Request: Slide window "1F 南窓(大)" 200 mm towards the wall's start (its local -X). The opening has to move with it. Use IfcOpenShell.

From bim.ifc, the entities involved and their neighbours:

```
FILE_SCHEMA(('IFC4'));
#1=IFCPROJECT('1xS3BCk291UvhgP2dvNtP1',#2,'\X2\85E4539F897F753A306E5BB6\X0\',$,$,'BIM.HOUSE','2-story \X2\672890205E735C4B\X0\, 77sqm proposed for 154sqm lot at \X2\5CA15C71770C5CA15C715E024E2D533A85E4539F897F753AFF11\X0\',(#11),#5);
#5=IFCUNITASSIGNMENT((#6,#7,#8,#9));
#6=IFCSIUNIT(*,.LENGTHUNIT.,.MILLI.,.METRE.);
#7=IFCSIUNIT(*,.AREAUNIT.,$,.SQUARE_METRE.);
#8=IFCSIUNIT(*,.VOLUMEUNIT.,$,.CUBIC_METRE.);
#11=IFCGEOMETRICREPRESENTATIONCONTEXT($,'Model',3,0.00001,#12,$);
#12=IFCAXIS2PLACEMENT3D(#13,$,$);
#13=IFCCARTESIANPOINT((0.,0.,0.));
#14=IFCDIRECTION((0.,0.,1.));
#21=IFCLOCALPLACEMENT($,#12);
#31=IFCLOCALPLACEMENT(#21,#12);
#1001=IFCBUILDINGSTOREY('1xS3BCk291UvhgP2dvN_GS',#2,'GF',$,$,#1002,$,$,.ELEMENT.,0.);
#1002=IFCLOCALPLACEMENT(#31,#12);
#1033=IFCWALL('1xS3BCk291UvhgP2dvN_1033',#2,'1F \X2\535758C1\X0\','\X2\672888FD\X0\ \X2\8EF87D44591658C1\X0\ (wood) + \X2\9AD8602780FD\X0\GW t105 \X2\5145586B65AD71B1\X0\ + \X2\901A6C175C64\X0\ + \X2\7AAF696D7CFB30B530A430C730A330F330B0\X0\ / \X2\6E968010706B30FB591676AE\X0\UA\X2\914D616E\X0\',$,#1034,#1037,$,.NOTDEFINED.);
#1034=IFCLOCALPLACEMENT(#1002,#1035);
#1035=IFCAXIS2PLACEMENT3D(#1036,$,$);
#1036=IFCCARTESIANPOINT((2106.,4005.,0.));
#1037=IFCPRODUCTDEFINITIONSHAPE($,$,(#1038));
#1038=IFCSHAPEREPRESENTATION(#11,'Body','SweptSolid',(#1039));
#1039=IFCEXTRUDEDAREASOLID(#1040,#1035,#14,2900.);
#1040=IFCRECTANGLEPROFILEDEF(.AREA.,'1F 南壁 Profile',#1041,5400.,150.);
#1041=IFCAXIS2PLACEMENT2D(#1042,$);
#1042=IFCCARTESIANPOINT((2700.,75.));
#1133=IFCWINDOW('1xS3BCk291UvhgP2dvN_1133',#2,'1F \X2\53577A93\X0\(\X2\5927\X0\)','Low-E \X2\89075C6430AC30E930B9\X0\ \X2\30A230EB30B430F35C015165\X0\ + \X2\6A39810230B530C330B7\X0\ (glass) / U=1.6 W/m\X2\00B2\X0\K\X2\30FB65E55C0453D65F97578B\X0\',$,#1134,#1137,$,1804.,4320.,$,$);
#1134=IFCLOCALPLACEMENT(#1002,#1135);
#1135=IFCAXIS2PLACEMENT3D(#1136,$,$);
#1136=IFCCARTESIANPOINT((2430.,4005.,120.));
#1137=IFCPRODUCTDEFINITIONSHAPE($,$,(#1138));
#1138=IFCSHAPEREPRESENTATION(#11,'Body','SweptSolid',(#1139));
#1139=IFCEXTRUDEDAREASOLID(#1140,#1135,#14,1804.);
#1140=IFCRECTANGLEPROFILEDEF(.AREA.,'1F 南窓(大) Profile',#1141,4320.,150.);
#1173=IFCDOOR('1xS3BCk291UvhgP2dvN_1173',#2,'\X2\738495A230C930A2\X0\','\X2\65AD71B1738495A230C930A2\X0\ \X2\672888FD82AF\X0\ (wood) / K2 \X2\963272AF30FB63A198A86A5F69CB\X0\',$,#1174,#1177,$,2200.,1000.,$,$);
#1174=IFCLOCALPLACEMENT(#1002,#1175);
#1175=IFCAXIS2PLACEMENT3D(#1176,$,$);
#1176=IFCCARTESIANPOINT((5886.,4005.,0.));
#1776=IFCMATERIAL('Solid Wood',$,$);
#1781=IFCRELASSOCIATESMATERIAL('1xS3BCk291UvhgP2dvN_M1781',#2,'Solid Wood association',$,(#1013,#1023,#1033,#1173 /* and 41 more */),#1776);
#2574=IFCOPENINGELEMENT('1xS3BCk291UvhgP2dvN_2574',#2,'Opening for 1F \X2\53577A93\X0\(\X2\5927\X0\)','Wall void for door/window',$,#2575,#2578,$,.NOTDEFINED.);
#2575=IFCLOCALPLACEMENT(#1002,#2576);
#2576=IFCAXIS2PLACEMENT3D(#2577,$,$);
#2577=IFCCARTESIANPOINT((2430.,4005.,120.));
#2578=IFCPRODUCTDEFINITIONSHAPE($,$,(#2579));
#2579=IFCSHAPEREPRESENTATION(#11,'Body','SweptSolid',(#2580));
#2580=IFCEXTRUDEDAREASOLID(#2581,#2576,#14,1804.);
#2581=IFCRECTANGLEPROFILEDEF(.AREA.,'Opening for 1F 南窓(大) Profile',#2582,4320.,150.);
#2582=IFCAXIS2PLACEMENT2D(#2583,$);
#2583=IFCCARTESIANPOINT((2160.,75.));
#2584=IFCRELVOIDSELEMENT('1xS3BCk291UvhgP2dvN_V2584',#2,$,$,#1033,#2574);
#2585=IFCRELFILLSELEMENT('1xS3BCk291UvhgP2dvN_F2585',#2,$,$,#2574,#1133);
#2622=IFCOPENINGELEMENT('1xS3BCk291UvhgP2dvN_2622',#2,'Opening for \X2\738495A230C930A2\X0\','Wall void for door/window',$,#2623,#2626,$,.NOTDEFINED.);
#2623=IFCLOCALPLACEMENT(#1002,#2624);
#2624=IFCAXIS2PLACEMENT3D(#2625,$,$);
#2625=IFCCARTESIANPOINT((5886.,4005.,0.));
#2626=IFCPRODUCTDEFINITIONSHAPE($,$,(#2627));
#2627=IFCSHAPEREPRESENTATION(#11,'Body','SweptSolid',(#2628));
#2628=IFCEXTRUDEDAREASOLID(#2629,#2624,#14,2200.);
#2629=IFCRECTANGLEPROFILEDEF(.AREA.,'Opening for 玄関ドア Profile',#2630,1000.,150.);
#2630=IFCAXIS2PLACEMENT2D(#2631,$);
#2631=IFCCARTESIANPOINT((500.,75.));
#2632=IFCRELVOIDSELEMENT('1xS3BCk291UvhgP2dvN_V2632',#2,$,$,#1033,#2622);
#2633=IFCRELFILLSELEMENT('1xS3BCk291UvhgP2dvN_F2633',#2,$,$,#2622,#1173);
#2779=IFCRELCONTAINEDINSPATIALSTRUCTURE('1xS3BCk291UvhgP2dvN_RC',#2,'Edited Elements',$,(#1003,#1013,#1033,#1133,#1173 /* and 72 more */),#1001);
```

```python
import ifcopenshell
import ifcopenshell.api.geometry
import ifcopenshell.util.placement

model = ifcopenshell.open("bim.ifc")

window = model.by_guid("1xS3BCk291UvhgP2dvN_1133")
opening = window.FillsVoids[0].RelatingOpeningElement
wall = opening.VoidsElements[0].RelatingBuildingElement

wall_matrix = ifcopenshell.util.placement.get_local_placement(wall.ObjectPlacement)
shift = wall_matrix[:3, 0] * -200.0
before = ifcopenshell.util.placement.get_local_placement(window.ObjectPlacement)[:3, 3].copy()

# The window is not placed relative to its opening, so move both.
for product in (opening, window):
    matrix = ifcopenshell.util.placement.get_local_placement(product.ObjectPlacement)
    matrix[:3, 3] += shift
    ifcopenshell.api.geometry.edit_object_placement(model, product=product, matrix=matrix, is_si=False)

after = ifcopenshell.util.placement.get_local_placement(window.ObjectPlacement)[:3, 3]
print("window moved by", (after - before).round(3) + 0.0)

model.write("bim_edited.ifc")
```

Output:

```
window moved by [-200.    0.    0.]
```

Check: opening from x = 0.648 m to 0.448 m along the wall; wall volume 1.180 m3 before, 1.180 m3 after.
